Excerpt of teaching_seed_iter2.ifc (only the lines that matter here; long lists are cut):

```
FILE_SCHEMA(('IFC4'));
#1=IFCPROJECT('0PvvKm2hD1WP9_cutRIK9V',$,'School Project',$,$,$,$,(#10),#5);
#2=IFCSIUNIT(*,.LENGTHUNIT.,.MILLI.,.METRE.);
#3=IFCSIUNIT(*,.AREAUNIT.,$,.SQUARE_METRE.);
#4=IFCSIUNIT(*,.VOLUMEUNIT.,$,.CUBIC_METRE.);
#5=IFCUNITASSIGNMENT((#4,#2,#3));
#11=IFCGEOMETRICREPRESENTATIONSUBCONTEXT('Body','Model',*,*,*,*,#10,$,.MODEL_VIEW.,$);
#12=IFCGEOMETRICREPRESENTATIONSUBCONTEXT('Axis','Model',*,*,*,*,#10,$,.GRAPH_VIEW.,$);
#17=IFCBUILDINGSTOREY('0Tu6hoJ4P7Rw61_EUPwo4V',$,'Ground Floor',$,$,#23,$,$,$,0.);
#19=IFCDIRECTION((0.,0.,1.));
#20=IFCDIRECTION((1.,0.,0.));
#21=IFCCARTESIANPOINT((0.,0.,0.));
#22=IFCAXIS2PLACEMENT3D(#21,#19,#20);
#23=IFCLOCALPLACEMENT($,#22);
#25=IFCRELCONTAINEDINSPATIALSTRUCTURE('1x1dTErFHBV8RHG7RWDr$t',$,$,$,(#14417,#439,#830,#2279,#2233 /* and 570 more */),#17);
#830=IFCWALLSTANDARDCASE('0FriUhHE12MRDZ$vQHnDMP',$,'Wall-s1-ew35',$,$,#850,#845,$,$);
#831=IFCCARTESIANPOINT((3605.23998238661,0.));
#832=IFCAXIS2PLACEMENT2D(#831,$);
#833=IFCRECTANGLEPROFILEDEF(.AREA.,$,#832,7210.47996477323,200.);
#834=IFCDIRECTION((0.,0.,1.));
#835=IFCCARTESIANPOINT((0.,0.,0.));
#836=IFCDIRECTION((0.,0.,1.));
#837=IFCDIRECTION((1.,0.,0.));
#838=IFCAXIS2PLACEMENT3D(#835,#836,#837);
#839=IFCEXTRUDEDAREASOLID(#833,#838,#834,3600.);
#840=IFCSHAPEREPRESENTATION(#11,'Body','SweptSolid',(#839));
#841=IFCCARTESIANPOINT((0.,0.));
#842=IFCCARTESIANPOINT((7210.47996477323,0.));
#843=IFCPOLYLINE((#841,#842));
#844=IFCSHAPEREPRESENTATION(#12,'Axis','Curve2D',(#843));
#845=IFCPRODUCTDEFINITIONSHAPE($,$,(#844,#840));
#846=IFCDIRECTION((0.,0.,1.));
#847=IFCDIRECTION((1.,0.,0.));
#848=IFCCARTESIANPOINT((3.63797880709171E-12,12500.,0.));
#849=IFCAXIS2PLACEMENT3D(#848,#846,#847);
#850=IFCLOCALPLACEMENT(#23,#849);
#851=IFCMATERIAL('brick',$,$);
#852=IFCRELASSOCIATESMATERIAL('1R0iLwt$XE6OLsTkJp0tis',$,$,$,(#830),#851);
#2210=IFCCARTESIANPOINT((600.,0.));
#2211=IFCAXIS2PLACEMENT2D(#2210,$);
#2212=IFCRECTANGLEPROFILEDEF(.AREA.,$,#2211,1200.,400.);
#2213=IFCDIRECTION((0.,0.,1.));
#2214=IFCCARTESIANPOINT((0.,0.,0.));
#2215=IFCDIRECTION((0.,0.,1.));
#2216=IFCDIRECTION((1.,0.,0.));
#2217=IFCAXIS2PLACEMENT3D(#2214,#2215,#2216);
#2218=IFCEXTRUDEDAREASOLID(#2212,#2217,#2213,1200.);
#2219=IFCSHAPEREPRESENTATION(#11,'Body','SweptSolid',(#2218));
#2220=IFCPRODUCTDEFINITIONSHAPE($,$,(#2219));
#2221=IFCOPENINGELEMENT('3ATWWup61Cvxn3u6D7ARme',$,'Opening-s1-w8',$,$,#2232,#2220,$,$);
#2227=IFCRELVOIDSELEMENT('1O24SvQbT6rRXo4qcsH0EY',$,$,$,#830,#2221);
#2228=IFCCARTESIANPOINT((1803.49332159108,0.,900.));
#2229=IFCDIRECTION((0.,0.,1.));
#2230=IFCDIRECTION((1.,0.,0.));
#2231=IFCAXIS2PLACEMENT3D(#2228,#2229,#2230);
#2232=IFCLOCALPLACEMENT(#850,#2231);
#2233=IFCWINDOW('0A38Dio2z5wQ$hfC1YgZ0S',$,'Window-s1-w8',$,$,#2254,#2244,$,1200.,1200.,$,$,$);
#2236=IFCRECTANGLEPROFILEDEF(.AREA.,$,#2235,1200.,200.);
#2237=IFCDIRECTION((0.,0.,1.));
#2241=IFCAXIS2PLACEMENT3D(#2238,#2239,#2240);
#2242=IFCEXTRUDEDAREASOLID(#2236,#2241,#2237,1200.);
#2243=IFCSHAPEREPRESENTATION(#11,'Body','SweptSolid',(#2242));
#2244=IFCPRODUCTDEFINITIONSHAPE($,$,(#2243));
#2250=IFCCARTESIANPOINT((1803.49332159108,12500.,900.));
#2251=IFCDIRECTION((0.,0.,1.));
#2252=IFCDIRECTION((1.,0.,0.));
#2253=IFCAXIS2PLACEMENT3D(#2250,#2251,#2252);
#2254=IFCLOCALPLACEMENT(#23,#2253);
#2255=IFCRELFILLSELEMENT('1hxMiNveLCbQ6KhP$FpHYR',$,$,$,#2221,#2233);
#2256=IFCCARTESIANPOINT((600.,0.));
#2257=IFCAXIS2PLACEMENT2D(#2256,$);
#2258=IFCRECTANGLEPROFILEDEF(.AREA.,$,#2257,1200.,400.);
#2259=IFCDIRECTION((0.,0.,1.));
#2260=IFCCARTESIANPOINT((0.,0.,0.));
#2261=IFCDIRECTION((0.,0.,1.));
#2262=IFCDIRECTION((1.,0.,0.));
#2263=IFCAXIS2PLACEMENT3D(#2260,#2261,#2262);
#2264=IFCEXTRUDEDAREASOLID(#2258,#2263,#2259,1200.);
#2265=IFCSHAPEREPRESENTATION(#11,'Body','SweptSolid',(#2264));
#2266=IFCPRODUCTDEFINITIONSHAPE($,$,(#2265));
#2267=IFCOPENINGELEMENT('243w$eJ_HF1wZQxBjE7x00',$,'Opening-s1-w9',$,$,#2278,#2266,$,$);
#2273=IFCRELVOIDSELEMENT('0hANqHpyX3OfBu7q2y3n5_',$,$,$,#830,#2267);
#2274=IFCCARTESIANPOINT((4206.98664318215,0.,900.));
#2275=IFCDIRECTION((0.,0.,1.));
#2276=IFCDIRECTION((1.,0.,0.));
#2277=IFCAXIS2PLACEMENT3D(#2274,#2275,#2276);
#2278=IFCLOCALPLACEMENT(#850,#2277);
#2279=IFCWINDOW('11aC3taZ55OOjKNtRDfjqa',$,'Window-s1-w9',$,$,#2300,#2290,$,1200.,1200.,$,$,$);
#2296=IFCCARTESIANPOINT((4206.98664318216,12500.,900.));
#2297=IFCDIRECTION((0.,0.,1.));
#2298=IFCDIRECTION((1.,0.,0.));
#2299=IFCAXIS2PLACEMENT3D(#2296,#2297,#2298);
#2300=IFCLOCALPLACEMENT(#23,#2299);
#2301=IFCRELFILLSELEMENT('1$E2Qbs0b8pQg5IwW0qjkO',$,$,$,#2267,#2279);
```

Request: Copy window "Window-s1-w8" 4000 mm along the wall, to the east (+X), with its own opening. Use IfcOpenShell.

```python
import ifcopenshell
import ifcopenshell.api.feature
import ifcopenshell.api.geometry
import ifcopenshell.api.root
import ifcopenshell.geom
import ifcopenshell.util.element
import ifcopenshell.util.placement
import ifcopenshell.util.shape

model = ifcopenshell.open("teaching_seed_iter2.ifc")
settings = ifcopenshell.geom.settings()


def volume(element):
    """Net volume in cubic metres, openings subtracted."""
    shape = ifcopenshell.geom.create_shape(settings, element)
    return ifcopenshell.util.shape.get_volume(shape.geometry)


window = model.by_guid("0A38Dio2z5wQ$hfC1YgZ0S")
opening = window.FillsVoids[0].RelatingOpeningElement
wall = opening.VoidsElements[0].RelatingBuildingElement
before = volume(wall)
shift = ifcopenshell.util.placement.get_local_placement(wall.ObjectPlacement)[:3, 0] * 4000.0

# copy_class copies the void relationship, type, container and properties, but no geometry.
new_opening = ifcopenshell.api.root.copy_class(model, product=opening)
new_opening.Representation = ifcopenshell.util.element.copy_deep(
    model, opening.Representation, exclude=["IfcGeometricRepresentationContext", "IfcRepresentationMap"]
)
new_window = ifcopenshell.api.root.copy_class(model, product=window)
new_window.Representation = ifcopenshell.util.element.copy_deep(
    model, window.Representation, exclude=["IfcGeometricRepresentationContext", "IfcRepresentationMap"]
)
ifcopenshell.api.feature.add_filling(model, opening=new_opening, element=new_window)

for old, new in ((opening, new_opening), (window, new_window)):
    matrix = ifcopenshell.util.placement.get_local_placement(old.ObjectPlacement)
    matrix[:3, 3] += shift
    ifcopenshell.api.geometry.edit_object_placement(model, product=new, matrix=matrix, is_si=False)

after = volume(wall)

print(f"wall volume {before:.3f} -> {after:.3f} m3")

model.write("teaching_seed_iter2_edited.ifc")
```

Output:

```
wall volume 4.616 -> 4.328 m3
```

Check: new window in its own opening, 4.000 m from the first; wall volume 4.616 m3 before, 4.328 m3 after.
